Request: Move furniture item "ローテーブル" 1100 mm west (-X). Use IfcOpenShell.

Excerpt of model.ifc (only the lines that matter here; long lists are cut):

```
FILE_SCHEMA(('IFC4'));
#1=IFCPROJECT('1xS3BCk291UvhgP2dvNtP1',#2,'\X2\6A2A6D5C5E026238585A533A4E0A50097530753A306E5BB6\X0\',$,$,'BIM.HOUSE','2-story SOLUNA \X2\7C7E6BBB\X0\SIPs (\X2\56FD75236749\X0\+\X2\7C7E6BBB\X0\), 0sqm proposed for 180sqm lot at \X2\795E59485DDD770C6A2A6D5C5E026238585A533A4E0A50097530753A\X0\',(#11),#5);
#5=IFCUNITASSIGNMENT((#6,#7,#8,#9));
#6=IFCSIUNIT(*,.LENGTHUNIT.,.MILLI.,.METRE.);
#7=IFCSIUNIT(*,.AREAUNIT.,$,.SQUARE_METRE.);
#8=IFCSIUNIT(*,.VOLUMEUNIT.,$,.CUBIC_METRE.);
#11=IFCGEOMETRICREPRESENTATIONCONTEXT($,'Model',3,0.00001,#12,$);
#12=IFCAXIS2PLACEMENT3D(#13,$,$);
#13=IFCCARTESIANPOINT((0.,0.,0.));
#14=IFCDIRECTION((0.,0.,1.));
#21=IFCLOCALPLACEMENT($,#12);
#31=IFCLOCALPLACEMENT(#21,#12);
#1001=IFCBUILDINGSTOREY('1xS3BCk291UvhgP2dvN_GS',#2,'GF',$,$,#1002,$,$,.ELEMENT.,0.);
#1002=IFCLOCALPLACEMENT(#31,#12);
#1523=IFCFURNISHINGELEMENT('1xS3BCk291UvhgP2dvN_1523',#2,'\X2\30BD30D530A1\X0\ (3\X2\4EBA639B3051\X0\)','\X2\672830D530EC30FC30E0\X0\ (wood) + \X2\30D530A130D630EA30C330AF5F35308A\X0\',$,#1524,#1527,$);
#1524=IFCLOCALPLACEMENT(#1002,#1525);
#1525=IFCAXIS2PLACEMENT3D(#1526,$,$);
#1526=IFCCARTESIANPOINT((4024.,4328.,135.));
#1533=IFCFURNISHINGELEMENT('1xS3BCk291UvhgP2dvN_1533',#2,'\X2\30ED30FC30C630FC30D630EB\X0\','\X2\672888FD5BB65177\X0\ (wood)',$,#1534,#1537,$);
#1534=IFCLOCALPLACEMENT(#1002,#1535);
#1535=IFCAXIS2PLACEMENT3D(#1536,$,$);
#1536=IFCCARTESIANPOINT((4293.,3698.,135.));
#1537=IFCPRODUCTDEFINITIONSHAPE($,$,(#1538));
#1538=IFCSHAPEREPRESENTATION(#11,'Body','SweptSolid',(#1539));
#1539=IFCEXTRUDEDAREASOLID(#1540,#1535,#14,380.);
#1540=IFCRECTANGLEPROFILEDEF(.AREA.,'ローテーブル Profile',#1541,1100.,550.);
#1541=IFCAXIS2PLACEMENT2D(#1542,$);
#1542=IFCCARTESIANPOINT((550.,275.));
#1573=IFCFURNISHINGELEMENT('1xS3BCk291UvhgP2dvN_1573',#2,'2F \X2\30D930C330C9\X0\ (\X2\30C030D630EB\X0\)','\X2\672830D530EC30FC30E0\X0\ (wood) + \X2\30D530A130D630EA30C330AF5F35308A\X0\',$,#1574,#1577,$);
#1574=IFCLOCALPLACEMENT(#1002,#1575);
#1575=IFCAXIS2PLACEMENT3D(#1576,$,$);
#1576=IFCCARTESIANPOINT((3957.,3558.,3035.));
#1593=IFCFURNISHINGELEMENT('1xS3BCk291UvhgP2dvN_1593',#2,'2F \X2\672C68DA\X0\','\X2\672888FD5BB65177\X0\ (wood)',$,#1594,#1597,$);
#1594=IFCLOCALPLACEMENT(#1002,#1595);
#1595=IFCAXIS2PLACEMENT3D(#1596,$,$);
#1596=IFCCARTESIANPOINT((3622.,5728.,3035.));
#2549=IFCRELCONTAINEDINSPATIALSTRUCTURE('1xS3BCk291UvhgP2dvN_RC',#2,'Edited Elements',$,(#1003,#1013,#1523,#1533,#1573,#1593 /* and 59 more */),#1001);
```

```python
import ifcopenshell
import ifcopenshell.api.geometry
import ifcopenshell.util.placement

model = ifcopenshell.open("model.ifc")

item = model.by_guid("1xS3BCk291UvhgP2dvN_1533")
matrix = ifcopenshell.util.placement.get_local_placement(item.ObjectPlacement)
matrix[0, 3] -= 1100.0
ifcopenshell.api.geometry.edit_object_placement(model, product=item, matrix=matrix, is_si=False)

print(ifcopenshell.util.placement.get_local_placement(item.ObjectPlacement).round(3) + 0.0)

model.write("model_rev.ifc")
```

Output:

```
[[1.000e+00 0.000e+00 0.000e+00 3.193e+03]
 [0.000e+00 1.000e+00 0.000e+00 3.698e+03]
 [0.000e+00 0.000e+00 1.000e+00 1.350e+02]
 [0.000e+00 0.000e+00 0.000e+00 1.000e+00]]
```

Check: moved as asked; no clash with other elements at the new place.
